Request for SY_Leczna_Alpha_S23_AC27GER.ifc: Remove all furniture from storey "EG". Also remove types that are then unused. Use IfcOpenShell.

First a look at what the model holds.

```python
import ifcopenshell
import ifcopenshell.util.element

model = ifcopenshell.open("SY_Leczna_Alpha_S23_AC27GER.ifc")
print(model.schema)
storey = next(s for s in model.by_type("IfcBuildingStorey") if s.Name == "EG")
furniture = [e for e in ifcopenshell.util.element.get_decomposition(storey) if e.is_a("IfcFurnishingElement")]
seen = {}
for e in furniture:
    element_type = ifcopenshell.util.element.get_type(e)
    name = element_type.Name if element_type not in (None, e) else None
    seen[name] = seen.get(name, 0) + 1
for name, count in sorted(seen.items(), key=str):
    print(count, "x", name)
```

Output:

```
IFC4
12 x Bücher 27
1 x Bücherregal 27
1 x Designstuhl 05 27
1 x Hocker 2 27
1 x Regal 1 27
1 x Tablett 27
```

```python
import ifcopenshell
import ifcopenshell.api.root
import ifcopenshell.util.element

model = ifcopenshell.open("SY_Leczna_Alpha_S23_AC27GER.ifc")

storey = next(s for s in model.by_type("IfcBuildingStorey") if s.Name == "EG")
furniture = [e for e in ifcopenshell.util.element.get_decomposition(storey) if e.is_a("IfcFurnishingElement")]
types = {ifcopenshell.util.element.get_type(e) for e in furniture} - {None, *furniture}

for e in furniture:
    ifcopenshell.api.root.remove_product(model, product=e)
print(len(furniture), "removed")

unused = [t for t in types if not ifcopenshell.util.element.get_types(t)]
for t in unused:
    ifcopenshell.api.root.remove_product(model, product=t)
print(len(unused), "unused types removed")

model.write("SY_Leczna_Alpha_S23_AC27GER_rev.ifc")
```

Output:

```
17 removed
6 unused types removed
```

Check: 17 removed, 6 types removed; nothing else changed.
